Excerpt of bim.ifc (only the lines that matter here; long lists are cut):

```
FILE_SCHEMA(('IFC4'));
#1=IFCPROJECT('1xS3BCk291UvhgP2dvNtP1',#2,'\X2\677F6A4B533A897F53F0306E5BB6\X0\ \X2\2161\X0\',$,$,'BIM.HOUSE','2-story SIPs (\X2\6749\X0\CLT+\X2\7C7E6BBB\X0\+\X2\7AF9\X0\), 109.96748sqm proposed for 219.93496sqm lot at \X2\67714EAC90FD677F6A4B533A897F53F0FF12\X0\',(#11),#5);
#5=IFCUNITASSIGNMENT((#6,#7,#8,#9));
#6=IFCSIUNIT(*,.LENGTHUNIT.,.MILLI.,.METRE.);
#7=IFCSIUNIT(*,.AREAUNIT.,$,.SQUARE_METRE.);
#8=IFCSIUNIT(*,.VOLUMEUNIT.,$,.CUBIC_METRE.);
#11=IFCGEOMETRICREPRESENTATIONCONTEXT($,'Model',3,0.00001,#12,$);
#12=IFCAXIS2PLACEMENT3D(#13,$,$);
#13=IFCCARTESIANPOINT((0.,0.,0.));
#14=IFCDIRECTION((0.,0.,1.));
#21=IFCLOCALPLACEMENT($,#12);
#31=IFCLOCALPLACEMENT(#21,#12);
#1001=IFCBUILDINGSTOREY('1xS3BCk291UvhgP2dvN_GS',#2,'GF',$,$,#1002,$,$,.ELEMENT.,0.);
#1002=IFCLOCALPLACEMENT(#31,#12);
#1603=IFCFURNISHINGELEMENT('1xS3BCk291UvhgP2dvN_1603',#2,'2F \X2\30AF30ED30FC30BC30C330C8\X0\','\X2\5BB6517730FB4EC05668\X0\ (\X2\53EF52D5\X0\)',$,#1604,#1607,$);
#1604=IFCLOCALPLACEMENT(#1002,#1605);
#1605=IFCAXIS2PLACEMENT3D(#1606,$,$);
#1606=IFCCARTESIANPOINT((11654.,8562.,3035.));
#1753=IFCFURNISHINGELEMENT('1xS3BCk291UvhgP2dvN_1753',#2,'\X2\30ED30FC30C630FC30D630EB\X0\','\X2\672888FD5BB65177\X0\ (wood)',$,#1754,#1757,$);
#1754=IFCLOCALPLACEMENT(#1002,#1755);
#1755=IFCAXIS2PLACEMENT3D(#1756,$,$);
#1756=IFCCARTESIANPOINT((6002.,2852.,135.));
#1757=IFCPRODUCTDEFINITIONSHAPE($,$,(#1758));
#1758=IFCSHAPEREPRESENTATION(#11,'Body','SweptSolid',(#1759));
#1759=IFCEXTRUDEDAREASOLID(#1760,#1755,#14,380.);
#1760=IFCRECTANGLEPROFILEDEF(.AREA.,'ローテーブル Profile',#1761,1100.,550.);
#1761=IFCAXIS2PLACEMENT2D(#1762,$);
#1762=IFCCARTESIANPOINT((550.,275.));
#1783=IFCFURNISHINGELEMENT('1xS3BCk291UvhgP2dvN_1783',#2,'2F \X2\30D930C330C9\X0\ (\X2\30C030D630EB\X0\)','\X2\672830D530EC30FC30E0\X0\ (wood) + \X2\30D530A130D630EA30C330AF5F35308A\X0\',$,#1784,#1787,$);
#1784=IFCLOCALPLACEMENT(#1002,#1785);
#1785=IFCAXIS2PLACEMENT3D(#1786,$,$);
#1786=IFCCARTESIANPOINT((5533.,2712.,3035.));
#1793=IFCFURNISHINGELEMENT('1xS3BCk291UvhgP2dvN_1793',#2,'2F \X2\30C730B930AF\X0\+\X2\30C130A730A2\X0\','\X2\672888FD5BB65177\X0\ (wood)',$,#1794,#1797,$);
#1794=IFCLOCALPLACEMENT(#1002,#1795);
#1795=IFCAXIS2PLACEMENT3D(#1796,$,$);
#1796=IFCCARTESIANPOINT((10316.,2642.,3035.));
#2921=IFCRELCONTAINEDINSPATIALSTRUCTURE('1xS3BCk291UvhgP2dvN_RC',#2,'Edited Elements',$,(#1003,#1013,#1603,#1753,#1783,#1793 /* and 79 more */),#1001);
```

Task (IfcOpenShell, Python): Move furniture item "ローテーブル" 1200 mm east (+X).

```python
import ifcopenshell
import ifcopenshell.api.geometry
import ifcopenshell.util.placement

model = ifcopenshell.open("bim.ifc")

item = model.by_guid("1xS3BCk291UvhgP2dvN_1753")
matrix = ifcopenshell.util.placement.get_local_placement(item.ObjectPlacement)
matrix[0, 3] += 1200.0
ifcopenshell.api.geometry.edit_object_placement(model, product=item, matrix=matrix, is_si=False)

print(ifcopenshell.util.placement.get_local_placement(item.ObjectPlacement).round(3) + 0.0)

model.write("bim_edited.ifc")
```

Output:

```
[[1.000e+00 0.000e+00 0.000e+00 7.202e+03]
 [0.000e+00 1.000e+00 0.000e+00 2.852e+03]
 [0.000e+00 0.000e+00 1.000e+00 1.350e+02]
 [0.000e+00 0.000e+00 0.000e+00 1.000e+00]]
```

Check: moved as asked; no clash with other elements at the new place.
